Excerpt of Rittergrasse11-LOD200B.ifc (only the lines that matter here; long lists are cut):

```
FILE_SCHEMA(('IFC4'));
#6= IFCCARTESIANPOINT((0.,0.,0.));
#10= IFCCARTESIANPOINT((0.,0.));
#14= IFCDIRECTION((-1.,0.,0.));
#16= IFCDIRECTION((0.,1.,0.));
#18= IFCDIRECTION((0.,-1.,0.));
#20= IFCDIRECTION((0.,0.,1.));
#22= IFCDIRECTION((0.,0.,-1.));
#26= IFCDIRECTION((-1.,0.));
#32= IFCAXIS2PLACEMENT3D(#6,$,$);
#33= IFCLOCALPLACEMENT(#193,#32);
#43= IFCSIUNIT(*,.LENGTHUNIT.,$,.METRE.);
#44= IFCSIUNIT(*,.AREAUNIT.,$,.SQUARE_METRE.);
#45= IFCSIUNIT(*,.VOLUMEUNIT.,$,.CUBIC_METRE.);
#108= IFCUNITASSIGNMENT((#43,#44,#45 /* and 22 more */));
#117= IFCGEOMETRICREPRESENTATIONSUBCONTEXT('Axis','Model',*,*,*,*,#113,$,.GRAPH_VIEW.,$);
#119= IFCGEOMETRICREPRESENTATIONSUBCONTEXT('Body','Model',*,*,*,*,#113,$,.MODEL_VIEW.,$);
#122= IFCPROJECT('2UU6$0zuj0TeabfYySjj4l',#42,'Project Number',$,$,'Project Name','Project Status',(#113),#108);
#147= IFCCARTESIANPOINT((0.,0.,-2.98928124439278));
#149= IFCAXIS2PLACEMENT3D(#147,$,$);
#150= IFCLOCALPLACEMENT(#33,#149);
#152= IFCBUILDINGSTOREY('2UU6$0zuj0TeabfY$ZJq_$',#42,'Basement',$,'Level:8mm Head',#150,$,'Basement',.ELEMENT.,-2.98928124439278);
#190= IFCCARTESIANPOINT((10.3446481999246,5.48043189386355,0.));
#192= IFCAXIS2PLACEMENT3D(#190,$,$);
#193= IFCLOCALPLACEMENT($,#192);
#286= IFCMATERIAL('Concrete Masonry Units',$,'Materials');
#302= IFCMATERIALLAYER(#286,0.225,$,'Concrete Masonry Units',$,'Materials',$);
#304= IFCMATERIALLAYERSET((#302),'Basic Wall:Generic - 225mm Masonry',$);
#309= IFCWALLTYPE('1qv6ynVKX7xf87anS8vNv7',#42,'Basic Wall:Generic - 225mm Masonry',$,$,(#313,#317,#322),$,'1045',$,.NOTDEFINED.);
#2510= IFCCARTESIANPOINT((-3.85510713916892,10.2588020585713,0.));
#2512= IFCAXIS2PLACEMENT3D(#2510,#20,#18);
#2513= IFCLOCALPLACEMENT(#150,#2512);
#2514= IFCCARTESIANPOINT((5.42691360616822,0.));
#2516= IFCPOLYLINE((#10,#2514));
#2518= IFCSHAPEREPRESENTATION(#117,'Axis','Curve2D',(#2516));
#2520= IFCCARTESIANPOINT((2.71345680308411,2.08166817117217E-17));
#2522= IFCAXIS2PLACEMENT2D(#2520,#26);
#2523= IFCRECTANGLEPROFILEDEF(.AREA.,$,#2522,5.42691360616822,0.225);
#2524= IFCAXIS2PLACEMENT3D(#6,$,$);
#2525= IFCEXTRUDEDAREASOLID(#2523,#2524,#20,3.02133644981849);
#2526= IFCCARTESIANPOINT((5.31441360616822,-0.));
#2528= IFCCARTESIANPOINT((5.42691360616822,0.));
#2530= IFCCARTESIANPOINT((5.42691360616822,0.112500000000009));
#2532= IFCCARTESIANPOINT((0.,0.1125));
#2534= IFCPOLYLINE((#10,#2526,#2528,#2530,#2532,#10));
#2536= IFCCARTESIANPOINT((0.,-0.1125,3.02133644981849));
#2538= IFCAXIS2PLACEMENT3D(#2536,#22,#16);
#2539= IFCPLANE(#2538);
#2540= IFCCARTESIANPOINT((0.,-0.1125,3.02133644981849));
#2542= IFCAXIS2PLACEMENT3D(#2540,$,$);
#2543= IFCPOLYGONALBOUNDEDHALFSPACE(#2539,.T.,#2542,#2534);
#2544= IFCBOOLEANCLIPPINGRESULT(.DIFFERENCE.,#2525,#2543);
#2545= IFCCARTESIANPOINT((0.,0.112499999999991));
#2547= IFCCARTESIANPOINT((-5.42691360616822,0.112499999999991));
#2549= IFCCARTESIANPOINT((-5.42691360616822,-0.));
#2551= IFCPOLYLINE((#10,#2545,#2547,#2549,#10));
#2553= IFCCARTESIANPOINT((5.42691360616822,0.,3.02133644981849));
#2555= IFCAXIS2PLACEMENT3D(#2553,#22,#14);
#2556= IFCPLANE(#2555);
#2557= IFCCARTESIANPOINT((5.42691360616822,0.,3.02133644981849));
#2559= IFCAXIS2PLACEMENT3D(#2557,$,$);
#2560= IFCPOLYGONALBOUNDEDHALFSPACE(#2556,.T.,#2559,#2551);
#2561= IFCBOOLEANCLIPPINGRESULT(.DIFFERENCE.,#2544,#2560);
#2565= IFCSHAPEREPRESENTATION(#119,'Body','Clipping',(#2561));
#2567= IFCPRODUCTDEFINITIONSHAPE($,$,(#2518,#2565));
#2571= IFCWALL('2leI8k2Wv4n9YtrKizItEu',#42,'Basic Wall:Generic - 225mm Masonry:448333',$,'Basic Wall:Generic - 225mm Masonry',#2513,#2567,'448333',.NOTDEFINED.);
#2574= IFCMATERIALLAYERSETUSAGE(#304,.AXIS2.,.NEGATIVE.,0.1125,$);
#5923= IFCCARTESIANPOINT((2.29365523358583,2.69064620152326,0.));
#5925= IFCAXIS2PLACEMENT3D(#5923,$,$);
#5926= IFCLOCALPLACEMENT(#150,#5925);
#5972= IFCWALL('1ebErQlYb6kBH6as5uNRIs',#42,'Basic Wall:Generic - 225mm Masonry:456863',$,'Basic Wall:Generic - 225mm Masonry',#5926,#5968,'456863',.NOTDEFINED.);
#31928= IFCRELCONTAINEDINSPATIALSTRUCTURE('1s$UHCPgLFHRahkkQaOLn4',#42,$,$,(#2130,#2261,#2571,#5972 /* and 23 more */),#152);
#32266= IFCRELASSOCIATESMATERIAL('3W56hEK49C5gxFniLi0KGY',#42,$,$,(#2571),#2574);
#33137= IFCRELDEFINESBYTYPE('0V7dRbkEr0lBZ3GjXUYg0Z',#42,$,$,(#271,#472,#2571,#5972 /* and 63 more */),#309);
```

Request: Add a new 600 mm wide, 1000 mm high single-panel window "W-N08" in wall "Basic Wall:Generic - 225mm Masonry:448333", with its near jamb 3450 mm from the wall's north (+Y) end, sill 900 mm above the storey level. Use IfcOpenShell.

```python
import numpy as np
import ifcopenshell
import ifcopenshell.api.feature
import ifcopenshell.api.geometry
import ifcopenshell.api.root
import ifcopenshell.api.spatial
import ifcopenshell.geom
import ifcopenshell.util.element
import ifcopenshell.util.placement
import ifcopenshell.util.representation
import ifcopenshell.util.shape
import ifcopenshell.util.unit

model = ifcopenshell.open("Rittergrasse11-LOD200B.ifc")
unit_scale = ifcopenshell.util.unit.calculate_unit_scale(model)
settings = ifcopenshell.geom.settings()


def volume(element):
    """Net volume in cubic metres, openings subtracted."""
    shape = ifcopenshell.geom.create_shape(settings, element)
    return ifcopenshell.util.shape.get_volume(shape.geometry)


wall = model.by_id(2571)
storey = ifcopenshell.util.element.get_container(wall, ifc_class="IfcBuildingStorey")
context = ifcopenshell.util.representation.get_context(model, "Model", "Body", "MODEL_VIEW")
before = volume(wall)

width, height, from_end, sill = 0.6, 1, 3.45, 0.9  # metres

# The wall runs along its own X axis, and the end named is its -X end.
wall_shape = ifcopenshell.geom.create_shape(settings, wall)
x, y, z = ifcopenshell.util.shape.get_vertices(wall_shape.geometry).T
start = x.min() + from_end
face, thickness = float(y.min()), float(y.max() - y.min())
wall_matrix = ifcopenshell.util.placement.get_local_placement(wall.ObjectPlacement)
level = ifcopenshell.util.placement.get_local_placement(storey.ObjectPlacement)[2, 3]


def in_wall(x, y):
    """Placement at x, y metres in the wall's axes, at sill height."""
    matrix = wall_matrix.copy()
    matrix[:, 3] = wall_matrix @ np.array([x / unit_scale, y / unit_scale, 0.0, 1.0])
    matrix[2, 3] = level + sill / unit_scale
    return matrix


# Opening: a box that overshoots both wall faces by 50 mm.
opening = ifcopenshell.api.root.create_entity(model, ifc_class="IfcOpeningElement", predefined_type="OPENING")
box = ifcopenshell.api.geometry.add_wall_representation(
    model, context=context, length=width, height=height, thickness=thickness + 0.1
)
ifcopenshell.api.geometry.assign_representation(model, product=opening, representation=box)
ifcopenshell.api.geometry.edit_object_placement(model, product=opening, matrix=in_wall(start, face - 0.05), is_si=False)
ifcopenshell.api.feature.add_feature(model, feature=opening, element=wall)

window = ifcopenshell.api.root.create_entity(model, ifc_class="IfcWindow", name="W-N08", predefined_type="WINDOW")
window.OverallWidth, window.OverallHeight = width / unit_scale, height / unit_scale
window.PartitioningType = "SINGLE_PANEL"
body = ifcopenshell.api.geometry.add_window_representation(
    model,
    context=context,
    overall_width=window.OverallWidth,
    overall_height=window.OverallHeight,
    partition_type="SINGLE_PANEL",
)
ifcopenshell.api.geometry.assign_representation(model, product=window, representation=body)
ifcopenshell.api.spatial.assign_container(model, products=[window], relating_structure=storey)
ifcopenshell.api.feature.add_filling(model, opening=opening, element=window)

# Centre the window in the wall's thickness.
ifcopenshell.api.geometry.edit_object_placement(model, product=window, matrix=in_wall(start, face), is_si=False)
window_shape = ifcopenshell.geom.create_shape(settings, window)
depth = ifcopenshell.util.shape.get_vertices(window_shape.geometry)[:, 1]
offset = face + thickness / 2 - (depth.min() + depth.max()) / 2
ifcopenshell.api.geometry.edit_object_placement(model, product=window, matrix=in_wall(start, offset), is_si=False)

after = volume(wall)

print(f"wall volume {before:.3f} -> {after:.3f} m3")

model.write("Rittergrasse11-LOD200B_updated.ifc")
```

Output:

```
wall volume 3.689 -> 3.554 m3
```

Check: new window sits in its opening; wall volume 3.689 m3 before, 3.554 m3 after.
